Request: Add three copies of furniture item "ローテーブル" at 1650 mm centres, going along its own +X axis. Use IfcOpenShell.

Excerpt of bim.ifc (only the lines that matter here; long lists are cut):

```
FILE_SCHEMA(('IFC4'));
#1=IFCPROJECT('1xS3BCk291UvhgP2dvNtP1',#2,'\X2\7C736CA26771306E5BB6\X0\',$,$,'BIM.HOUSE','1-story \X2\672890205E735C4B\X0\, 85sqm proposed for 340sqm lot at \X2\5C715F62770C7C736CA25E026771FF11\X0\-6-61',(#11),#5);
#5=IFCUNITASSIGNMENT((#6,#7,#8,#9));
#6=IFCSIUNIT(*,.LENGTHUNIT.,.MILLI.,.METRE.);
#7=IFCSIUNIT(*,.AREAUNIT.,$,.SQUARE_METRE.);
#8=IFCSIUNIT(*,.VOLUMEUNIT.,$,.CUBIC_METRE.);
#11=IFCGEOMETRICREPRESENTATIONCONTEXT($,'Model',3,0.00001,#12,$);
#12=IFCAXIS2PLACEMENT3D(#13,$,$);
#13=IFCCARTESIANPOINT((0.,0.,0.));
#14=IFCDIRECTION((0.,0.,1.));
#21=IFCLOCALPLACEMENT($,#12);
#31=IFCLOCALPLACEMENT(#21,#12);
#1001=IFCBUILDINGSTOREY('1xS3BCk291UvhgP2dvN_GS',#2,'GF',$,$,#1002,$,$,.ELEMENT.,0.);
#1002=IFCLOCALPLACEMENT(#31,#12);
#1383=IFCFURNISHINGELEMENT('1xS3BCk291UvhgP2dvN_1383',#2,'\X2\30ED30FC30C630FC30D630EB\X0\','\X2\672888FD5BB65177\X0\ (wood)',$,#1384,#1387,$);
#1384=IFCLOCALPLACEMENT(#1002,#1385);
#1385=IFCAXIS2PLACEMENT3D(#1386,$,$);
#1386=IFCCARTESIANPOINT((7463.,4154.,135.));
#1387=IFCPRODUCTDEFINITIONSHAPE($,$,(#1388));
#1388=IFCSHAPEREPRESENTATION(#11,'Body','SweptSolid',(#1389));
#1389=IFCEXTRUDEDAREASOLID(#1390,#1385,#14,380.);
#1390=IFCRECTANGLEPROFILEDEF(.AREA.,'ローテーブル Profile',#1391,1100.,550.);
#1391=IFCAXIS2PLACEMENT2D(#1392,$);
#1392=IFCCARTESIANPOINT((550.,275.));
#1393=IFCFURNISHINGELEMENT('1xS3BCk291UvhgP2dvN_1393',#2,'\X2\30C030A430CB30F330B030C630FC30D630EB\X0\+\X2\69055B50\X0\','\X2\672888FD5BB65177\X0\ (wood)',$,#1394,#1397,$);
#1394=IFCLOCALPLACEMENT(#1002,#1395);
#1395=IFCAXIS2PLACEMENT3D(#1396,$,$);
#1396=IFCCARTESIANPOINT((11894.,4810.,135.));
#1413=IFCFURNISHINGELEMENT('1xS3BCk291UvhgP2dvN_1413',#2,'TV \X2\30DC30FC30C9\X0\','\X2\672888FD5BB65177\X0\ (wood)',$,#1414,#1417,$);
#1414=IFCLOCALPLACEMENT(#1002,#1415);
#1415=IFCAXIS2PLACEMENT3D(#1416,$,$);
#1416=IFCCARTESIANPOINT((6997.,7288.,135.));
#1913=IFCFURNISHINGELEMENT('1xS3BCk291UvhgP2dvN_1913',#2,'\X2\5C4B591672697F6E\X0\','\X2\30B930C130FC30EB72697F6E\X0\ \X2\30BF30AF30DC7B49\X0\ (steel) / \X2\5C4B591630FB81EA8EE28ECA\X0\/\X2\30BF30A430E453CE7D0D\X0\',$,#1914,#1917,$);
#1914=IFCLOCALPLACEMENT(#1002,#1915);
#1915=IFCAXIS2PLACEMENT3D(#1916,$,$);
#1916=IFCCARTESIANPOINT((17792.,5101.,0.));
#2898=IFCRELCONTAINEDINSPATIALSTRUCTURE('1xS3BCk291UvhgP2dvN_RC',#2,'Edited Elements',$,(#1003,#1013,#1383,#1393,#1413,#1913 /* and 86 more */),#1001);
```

```python
import ifcopenshell
import ifcopenshell.api.geometry
import ifcopenshell.api.root
import ifcopenshell.util.element
import ifcopenshell.util.placement
import ifcopenshell.util.unit

model = ifcopenshell.open("bim.ifc")
unit_scale = ifcopenshell.util.unit.calculate_unit_scale(model)


def reuse_history(source, copy):
    """copy_class also copies each property set's owner history, people and application; keep the originals."""
    for rel in copy.IsDefinedBy:
        if rel.is_a("IfcRelDefinesByProperties") and (history := rel.RelatingPropertyDefinition.OwnerHistory):
            rel.RelatingPropertyDefinition.OwnerHistory = source.OwnerHistory
            ifcopenshell.util.element.remove_deep2(model, history)


source = model.by_guid("1xS3BCk291UvhgP2dvN_1383")
base = ifcopenshell.util.placement.get_local_placement(source.ObjectPlacement)
step = base[:3, 0] * 1.65 / unit_scale

for i in range(1, 4):
    copy = ifcopenshell.api.root.copy_class(model, product=source)
    copy.Representation = ifcopenshell.util.element.copy_deep(
        model, source.Representation, exclude=["IfcGeometricRepresentationContext", "IfcRepresentationMap"]
    )
    reuse_history(source, copy)
    matrix = base.copy()
    matrix[:3, 3] += i * step
    print("added at", matrix[:3, 3].round(3) + 0.0)
    ifcopenshell.api.geometry.edit_object_placement(model, product=copy, matrix=matrix, is_si=False)

model.write("bim_rev.ifc")
```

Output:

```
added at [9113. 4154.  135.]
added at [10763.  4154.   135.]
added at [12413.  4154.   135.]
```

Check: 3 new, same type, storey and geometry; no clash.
